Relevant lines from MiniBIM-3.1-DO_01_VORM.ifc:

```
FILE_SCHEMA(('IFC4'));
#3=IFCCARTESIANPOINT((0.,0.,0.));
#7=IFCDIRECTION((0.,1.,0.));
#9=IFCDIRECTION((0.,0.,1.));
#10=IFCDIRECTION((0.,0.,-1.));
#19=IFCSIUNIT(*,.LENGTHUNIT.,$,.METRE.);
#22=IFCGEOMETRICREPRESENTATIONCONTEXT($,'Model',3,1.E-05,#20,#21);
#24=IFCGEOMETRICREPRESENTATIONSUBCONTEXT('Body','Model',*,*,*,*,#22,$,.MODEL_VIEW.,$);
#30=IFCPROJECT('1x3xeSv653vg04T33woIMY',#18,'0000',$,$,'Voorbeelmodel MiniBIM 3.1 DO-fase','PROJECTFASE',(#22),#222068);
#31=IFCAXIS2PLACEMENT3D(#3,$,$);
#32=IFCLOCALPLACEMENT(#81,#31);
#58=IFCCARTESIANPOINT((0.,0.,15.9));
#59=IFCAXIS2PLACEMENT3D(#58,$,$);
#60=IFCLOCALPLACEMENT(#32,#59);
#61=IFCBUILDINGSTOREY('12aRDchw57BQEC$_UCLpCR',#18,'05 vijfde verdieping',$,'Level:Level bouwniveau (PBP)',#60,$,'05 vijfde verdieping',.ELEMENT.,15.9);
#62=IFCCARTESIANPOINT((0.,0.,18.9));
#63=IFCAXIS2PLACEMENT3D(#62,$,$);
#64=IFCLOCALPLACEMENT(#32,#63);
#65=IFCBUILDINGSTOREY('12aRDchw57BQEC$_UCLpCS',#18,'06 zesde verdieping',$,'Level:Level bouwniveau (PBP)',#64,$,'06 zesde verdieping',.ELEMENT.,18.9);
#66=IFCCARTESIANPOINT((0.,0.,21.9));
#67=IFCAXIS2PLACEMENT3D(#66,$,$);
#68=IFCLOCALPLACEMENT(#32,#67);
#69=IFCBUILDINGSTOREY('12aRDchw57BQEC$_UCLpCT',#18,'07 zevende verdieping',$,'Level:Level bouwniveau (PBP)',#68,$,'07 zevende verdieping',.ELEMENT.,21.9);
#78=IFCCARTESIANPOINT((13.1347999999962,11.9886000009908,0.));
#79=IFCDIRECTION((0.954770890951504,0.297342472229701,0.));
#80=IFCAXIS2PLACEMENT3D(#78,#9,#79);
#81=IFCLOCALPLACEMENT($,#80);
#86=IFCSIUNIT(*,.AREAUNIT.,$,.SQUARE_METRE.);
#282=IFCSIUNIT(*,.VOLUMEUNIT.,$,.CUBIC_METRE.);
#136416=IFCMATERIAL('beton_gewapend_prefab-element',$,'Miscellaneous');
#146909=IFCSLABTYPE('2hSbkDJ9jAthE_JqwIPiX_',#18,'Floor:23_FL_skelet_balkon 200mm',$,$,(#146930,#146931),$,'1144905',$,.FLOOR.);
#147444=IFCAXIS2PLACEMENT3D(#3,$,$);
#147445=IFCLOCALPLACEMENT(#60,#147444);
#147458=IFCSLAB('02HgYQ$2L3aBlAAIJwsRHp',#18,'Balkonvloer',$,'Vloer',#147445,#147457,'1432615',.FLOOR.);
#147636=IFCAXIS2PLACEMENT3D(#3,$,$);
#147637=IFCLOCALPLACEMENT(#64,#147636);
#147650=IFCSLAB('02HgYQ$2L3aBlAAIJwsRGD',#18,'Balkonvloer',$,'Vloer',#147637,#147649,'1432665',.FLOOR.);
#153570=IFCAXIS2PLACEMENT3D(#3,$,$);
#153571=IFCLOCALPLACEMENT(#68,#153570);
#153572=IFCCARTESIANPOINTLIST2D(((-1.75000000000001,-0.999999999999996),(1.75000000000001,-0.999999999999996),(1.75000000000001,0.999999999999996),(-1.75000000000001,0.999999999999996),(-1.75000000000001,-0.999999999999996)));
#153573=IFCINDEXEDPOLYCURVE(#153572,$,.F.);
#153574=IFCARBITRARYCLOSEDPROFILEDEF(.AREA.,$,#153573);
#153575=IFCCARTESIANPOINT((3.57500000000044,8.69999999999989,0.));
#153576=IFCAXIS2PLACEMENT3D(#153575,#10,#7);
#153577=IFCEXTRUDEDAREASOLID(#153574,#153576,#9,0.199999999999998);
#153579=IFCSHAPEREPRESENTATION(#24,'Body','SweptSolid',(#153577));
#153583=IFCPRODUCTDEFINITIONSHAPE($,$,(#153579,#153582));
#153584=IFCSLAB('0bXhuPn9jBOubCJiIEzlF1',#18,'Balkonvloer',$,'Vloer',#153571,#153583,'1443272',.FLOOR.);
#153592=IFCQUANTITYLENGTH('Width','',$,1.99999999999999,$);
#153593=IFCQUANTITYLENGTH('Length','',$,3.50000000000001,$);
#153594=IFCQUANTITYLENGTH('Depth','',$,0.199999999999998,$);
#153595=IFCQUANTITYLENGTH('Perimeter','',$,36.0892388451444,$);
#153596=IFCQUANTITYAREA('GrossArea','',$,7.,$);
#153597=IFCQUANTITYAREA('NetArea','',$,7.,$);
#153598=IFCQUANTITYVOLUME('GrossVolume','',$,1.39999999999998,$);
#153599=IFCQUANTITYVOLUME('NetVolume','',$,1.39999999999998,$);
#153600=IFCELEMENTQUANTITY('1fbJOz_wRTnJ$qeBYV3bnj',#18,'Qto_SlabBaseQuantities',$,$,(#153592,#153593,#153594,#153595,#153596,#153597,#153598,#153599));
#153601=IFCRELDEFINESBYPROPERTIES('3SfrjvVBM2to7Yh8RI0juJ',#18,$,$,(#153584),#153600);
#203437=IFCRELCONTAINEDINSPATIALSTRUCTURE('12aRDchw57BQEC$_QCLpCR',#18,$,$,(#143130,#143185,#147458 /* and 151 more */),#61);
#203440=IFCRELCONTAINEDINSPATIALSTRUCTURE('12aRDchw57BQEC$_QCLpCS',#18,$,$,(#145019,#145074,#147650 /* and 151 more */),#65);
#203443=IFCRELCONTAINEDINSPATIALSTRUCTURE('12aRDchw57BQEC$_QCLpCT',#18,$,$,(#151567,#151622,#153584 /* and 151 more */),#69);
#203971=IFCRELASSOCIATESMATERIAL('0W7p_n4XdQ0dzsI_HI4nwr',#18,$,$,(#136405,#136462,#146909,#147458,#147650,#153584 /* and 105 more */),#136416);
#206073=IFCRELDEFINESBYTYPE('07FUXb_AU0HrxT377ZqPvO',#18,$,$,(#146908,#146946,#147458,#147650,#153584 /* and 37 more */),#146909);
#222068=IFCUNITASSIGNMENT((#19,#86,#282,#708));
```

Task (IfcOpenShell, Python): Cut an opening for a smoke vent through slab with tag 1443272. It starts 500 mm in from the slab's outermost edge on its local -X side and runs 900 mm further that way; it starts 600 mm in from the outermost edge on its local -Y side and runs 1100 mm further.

```python
import numpy as np
import ifcopenshell
import ifcopenshell.api.feature
import ifcopenshell.api.geometry
import ifcopenshell.api.pset
import ifcopenshell.api.root
import ifcopenshell.geom
import ifcopenshell.util.element
import ifcopenshell.util.placement
import ifcopenshell.util.representation
import ifcopenshell.util.shape
import ifcopenshell.util.unit

model = ifcopenshell.open("MiniBIM-3.1-DO_01_VORM.ifc")
unit_scale = ifcopenshell.util.unit.calculate_unit_scale(model)
area_scale = ifcopenshell.util.unit.calculate_unit_scale(model, "AREAUNIT")
volume_scale = ifcopenshell.util.unit.calculate_unit_scale(model, "VOLUMEUNIT")
settings = ifcopenshell.geom.settings()


def volume(element):
    """Net volume in cubic metres, openings subtracted."""
    shape = ifcopenshell.geom.create_shape(settings, element)
    return ifcopenshell.util.shape.get_volume(shape.geometry)


slab = model.by_guid("0bXhuPn9jBOubCJiIEzlF1")
before = volume(slab)

# Extent in the slab's own axes, in metres. The edges named are its -X and -Y sides.
slab_shape = ifcopenshell.geom.create_shape(settings, slab)
vertices = ifcopenshell.util.shape.get_vertices(slab_shape.geometry)
x_min, y_min, bottom = vertices.min(axis=0)
top = vertices[:, 2].max()

opening = ifcopenshell.api.root.create_entity(model, ifc_class="IfcOpeningElement", name="Smoke vent opening", predefined_type="OPENING")
context = ifcopenshell.util.representation.get_context(model, "Model", "Body", "MODEL_VIEW")
width, depth = 0.9, 1.1
outline = [(0.0, 0.0), (width, 0.0), (width, depth), (0.0, depth), (0.0, 0.0)]
# Overshoot both faces by 50 mm so the cut is clean.
shape = ifcopenshell.api.geometry.add_slab_representation(
    model, context=context, depth=top - bottom + 0.1, polyline=outline
)
ifcopenshell.api.geometry.assign_representation(model, product=opening, representation=shape)

matrix = ifcopenshell.util.placement.get_local_placement(slab.ObjectPlacement)
matrix[:, 3] = matrix @ np.append(np.array([x_min + 0.5, y_min + 0.6, bottom - 0.05]) / unit_scale, 1.0)
ifcopenshell.api.geometry.edit_object_placement(model, product=opening, matrix=matrix, is_si=False)
ifcopenshell.api.feature.add_feature(model, feature=opening, element=slab)

after = volume(slab)

# Update the slab's stored quantities.
qto = model.by_id(ifcopenshell.util.element.get_pset(slab, "Qto_SlabBaseQuantities", should_inherit=False)["id"])
ifcopenshell.api.pset.edit_qto(model, qto=qto, properties={
    "NetArea": after / (top - bottom) / area_scale,
    "NetVolume": after / volume_scale,
})

print(f"slab volume {before:.3f} -> {after:.3f} m3")

model.write("MiniBIM-3.1-DO_01_VORM_rev.ifc")
```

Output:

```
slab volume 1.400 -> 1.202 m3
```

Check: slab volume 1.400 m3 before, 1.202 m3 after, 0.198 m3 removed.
